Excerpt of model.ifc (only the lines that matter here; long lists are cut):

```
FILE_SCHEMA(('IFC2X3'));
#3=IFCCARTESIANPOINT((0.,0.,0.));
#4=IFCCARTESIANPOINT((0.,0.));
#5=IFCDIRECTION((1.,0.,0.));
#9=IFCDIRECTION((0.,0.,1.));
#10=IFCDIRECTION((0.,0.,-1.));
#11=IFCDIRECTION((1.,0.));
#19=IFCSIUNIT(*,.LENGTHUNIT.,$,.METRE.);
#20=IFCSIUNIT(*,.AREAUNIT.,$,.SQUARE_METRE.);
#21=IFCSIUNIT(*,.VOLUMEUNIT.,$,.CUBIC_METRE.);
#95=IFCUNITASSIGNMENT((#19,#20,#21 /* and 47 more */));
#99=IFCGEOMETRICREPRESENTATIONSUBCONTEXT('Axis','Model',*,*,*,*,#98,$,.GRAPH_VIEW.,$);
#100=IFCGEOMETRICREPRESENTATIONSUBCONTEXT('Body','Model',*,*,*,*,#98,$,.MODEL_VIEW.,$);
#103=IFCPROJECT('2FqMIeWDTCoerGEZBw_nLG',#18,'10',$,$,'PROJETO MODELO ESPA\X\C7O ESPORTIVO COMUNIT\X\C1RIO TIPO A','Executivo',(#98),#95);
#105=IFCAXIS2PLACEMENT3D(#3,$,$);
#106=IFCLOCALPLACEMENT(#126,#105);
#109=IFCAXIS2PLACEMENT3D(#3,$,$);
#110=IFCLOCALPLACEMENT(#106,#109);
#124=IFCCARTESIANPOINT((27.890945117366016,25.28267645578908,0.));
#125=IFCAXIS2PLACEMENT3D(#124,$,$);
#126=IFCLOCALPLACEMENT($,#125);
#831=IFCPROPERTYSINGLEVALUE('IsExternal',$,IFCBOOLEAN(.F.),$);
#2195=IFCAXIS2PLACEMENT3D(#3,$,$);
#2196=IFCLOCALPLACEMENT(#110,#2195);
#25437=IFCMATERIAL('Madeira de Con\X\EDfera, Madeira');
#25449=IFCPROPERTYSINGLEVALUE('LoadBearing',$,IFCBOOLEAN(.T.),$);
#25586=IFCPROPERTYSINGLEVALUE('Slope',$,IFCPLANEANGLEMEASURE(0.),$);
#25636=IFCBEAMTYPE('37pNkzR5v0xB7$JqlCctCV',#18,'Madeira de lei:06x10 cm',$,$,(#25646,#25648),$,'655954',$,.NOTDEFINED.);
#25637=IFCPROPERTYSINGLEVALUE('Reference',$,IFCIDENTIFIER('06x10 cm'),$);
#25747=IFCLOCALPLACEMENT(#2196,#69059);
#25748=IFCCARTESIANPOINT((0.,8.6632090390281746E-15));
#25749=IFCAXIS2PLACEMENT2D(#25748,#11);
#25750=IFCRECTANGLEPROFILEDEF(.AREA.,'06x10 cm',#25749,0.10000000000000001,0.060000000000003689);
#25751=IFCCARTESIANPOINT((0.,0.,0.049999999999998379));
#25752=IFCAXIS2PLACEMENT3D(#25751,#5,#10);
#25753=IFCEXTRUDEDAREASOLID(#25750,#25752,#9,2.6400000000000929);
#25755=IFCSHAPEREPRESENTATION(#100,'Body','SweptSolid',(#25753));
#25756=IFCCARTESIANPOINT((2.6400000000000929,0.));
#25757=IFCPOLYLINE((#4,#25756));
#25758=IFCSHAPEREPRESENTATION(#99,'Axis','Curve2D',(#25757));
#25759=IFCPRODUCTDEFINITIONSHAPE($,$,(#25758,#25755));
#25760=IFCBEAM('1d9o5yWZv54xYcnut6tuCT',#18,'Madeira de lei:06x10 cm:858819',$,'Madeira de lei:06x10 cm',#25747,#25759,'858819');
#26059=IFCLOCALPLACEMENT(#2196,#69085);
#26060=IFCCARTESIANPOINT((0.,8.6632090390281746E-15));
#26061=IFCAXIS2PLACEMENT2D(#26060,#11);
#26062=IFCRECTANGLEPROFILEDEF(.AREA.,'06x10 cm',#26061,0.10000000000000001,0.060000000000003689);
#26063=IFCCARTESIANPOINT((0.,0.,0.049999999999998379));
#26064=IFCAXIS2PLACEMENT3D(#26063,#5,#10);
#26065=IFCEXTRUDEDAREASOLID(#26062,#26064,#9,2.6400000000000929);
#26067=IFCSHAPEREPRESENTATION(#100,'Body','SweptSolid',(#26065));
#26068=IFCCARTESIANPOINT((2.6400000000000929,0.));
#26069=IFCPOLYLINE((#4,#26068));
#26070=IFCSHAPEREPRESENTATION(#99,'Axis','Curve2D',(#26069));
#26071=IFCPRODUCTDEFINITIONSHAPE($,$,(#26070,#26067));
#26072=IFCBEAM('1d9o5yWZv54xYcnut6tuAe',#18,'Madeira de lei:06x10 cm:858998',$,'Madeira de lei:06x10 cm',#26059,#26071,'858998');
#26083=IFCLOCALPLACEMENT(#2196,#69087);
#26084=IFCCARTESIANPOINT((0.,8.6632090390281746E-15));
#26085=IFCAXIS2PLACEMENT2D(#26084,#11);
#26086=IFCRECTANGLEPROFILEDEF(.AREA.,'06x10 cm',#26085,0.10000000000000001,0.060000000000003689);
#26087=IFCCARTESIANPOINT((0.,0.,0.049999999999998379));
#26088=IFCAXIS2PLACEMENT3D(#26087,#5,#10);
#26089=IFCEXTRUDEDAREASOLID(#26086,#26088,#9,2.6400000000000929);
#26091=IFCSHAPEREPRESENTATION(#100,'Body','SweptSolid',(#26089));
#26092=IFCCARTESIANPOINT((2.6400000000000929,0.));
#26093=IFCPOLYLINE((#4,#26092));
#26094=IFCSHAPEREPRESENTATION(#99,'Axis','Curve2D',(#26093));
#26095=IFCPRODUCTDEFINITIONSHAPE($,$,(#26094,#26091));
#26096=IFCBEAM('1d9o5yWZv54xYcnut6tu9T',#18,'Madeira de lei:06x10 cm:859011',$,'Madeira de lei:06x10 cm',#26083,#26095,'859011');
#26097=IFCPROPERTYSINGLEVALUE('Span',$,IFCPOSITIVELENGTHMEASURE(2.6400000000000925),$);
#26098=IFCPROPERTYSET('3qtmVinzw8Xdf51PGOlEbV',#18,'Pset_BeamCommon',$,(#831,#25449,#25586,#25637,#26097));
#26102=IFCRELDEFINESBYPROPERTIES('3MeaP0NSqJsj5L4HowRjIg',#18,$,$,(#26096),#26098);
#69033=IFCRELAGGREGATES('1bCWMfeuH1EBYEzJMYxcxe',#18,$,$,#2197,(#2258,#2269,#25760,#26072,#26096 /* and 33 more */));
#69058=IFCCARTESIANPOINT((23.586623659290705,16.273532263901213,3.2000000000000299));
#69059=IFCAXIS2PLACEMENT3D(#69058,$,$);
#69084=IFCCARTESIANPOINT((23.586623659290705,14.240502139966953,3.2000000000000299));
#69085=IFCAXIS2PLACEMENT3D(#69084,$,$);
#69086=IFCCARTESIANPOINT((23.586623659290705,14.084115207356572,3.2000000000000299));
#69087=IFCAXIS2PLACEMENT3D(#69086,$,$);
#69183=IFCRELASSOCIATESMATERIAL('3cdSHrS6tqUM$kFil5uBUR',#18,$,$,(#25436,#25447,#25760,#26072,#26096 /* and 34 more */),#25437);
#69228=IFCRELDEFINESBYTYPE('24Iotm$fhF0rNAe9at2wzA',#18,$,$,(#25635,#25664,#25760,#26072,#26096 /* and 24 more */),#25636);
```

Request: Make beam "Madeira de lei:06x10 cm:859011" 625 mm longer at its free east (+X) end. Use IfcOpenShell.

```python
import numpy as np
import ifcopenshell
import ifcopenshell.api.pset
import ifcopenshell.util.element
import ifcopenshell.util.representation
import ifcopenshell.util.unit

model = ifcopenshell.open("model.ifc")
unit_scale = ifcopenshell.util.unit.calculate_unit_scale(model)

member = model.by_id(26096)
change = 0.625 / unit_scale

# The extrusion runs towards the end named, so only its depth changes.
body = ifcopenshell.util.representation.get_representation(member, "Model", "Body")
solid = body.Items[0]
old_length = solid.Depth
solid.Depth += change

# Move the axis end point with it.
axis = next(r for r in member.Representation.Representations if r.RepresentationIdentifier == "Axis").Items[0]
start, end = (np.array(p.Coordinates) for p in axis.Points)
end = end + (end - start) / np.linalg.norm(end - start) * change
point = model.createIfcCartesianPoint(end.tolist())
axis.Points = [axis.Points[0], point]

# Update the stored length and volume.
pset = model.by_id(ifcopenshell.util.element.get_pset(member, "Pset_BeamCommon", should_inherit=False)["id"])
ifcopenshell.api.pset.edit_pset(model, pset=pset, properties={
    "Span": model.create_entity("IfcPositiveLengthMeasure", solid.Depth),
})

print(f"length {old_length:g} -> {solid.Depth:g}")

model.write("model_v2.ifc")
```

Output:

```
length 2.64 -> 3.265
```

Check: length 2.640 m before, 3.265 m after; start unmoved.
